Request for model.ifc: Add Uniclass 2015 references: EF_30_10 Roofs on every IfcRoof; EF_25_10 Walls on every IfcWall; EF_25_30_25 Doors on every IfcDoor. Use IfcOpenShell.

First a look at what the model holds.

```python
import ifcopenshell

model = ifcopenshell.open("model.ifc")
print(model.schema)
print("classifications:", [c.Name for c in model.by_type("IfcClassification")])
for ifc_class in ("IfcDoor", "IfcRoof", "IfcStair", "IfcWall", "IfcWindow"):
    print(ifc_class, len(model.by_type(ifc_class)))
```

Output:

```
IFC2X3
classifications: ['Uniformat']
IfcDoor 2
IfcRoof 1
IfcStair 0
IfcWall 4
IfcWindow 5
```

```python
import ifcopenshell
import ifcopenshell.api.classification

model = ifcopenshell.open("model.ifc")

# IFC2X3 requires Source and Edition and has no link from the project to the system.
system = model.create_entity("IfcClassification", Source="NBS", Edition="2015", Name="Uniclass 2015")

codes = {
    "IfcRoof": ("EF_30_10", "Roofs"),
    "IfcWall": ("EF_25_10", "Walls"),
    "IfcDoor": ("EF_25_30_25", "Doors"),
}
for ifc_class, (code, name) in codes.items():
    products = model.by_type(ifc_class)
    ifcopenshell.api.classification.add_reference(
        model, products=products, classification=system, identification=code, name=name
    )
    print(code, len(products))

model.write("model-out.ifc")
```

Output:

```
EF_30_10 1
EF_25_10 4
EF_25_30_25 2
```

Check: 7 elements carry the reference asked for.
